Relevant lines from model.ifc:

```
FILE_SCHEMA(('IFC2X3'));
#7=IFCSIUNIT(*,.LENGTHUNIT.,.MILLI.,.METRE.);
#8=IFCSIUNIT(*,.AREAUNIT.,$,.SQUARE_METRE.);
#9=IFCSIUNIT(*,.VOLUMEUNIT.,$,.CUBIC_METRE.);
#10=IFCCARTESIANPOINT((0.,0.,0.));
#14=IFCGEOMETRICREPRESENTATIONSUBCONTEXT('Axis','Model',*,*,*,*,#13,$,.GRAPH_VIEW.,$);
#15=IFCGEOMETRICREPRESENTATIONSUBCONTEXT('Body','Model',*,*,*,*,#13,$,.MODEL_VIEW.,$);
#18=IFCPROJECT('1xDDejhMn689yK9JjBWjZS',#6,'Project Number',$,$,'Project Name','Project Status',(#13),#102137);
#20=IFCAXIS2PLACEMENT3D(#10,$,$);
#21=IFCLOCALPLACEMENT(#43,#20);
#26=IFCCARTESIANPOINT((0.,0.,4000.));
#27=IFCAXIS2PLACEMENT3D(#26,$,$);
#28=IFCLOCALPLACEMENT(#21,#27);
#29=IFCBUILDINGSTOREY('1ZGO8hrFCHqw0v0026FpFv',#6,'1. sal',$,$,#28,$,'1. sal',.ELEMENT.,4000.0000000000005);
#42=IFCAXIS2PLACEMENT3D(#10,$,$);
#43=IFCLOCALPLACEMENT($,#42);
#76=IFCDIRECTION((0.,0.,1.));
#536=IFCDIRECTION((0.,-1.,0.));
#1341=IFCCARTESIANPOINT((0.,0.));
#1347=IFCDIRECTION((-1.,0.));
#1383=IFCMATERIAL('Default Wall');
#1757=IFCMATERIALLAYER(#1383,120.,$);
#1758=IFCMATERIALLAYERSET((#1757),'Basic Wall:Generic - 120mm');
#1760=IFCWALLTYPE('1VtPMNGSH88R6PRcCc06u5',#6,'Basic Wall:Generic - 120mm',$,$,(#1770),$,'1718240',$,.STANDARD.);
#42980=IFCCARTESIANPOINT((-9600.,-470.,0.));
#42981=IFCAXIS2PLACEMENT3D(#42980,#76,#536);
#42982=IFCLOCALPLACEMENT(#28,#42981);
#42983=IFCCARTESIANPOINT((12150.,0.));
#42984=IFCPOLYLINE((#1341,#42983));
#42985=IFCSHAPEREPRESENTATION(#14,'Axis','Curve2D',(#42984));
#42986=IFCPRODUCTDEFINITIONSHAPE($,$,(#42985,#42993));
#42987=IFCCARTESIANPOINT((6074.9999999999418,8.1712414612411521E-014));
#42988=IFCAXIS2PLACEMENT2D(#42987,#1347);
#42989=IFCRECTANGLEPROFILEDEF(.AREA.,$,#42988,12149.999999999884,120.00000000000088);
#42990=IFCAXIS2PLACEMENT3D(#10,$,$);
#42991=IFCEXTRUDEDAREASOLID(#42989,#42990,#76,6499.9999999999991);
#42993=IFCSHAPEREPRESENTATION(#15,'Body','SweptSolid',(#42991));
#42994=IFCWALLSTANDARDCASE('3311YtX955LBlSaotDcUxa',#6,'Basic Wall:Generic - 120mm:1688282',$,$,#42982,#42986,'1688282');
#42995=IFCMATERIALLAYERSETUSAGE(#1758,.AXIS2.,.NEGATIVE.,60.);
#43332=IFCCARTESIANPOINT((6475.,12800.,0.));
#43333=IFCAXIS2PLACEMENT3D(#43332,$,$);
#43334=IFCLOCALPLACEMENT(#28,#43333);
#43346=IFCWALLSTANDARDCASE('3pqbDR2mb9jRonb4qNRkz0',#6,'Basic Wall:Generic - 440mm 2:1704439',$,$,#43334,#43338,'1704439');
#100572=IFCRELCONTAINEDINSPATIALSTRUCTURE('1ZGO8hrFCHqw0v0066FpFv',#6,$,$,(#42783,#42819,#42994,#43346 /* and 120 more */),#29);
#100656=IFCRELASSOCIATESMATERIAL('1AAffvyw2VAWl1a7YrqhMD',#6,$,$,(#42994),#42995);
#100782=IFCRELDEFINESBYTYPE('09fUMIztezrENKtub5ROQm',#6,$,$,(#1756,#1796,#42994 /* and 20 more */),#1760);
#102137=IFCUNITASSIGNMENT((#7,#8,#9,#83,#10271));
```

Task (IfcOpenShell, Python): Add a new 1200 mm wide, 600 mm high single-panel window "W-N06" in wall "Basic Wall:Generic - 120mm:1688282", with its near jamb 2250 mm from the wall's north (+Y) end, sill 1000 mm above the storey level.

```python
import numpy as np
import ifcopenshell
import ifcopenshell.api.feature
import ifcopenshell.api.geometry
import ifcopenshell.api.root
import ifcopenshell.api.spatial
import ifcopenshell.api.type
import ifcopenshell.geom
import ifcopenshell.util.element
import ifcopenshell.util.placement
import ifcopenshell.util.representation
import ifcopenshell.util.shape
import ifcopenshell.util.unit

model = ifcopenshell.open("model.ifc")
unit_scale = ifcopenshell.util.unit.calculate_unit_scale(model)
settings = ifcopenshell.geom.settings()


def volume(element):
    """Net volume in cubic metres, openings subtracted."""
    shape = ifcopenshell.geom.create_shape(settings, element)
    return ifcopenshell.util.shape.get_volume(shape.geometry)


wall = model.by_guid("3311YtX955LBlSaotDcUxa")
storey = ifcopenshell.util.element.get_container(wall, ifc_class="IfcBuildingStorey")
context = ifcopenshell.util.representation.get_context(model, "Model", "Body", "MODEL_VIEW")
before = volume(wall)

width, height, from_end, sill = 1.2, 0.6, 2.25, 1  # metres

# The wall runs along its own X axis, and the end named is its -X end.
wall_shape = ifcopenshell.geom.create_shape(settings, wall)
x, y, z = ifcopenshell.util.shape.get_vertices(wall_shape.geometry).T
start = x.min() + from_end
face, thickness = float(y.min()), float(y.max() - y.min())
wall_matrix = ifcopenshell.util.placement.get_local_placement(wall.ObjectPlacement)
level = ifcopenshell.util.placement.get_local_placement(storey.ObjectPlacement)[2, 3]


def in_wall(x, y):
    """Placement at x, y metres in the wall's axes, at sill height."""
    matrix = wall_matrix.copy()
    matrix[:, 3] = wall_matrix @ np.array([x / unit_scale, y / unit_scale, 0.0, 1.0])
    matrix[2, 3] = level + sill / unit_scale
    return matrix


# Opening: a box that overshoots both wall faces by 50 mm.
opening = ifcopenshell.api.root.create_entity(model, ifc_class="IfcOpeningElement")
box = ifcopenshell.api.geometry.add_wall_representation(
    model, context=context, length=width, height=height, thickness=thickness + 0.1
)
ifcopenshell.api.geometry.assign_representation(model, product=opening, representation=box)
ifcopenshell.api.geometry.edit_object_placement(model, product=opening, matrix=in_wall(start, face - 0.05), is_si=False)
ifcopenshell.api.feature.add_feature(model, feature=opening, element=wall)

window = ifcopenshell.api.root.create_entity(model, ifc_class="IfcWindow", name="W-N06")
window.OverallWidth, window.OverallHeight = width / unit_scale, height / unit_scale
body = ifcopenshell.api.geometry.add_window_representation(
    model,
    context=context,
    overall_width=window.OverallWidth,
    overall_height=window.OverallHeight,
    partition_type="SINGLE_PANEL",
)
ifcopenshell.api.geometry.assign_representation(model, product=window, representation=body)
ifcopenshell.api.spatial.assign_container(model, products=[window], relating_structure=storey)
fills = ifcopenshell.api.feature.add_filling(model, opening=opening, element=window)
fills.OwnerHistory = window.OwnerHistory  # required in IFC2X3

# IFC2X3 keeps the operation on the window style.
style = ifcopenshell.api.root.create_entity(model, ifc_class="IfcWindowStyle", name="W-N06")
style.OperationType, style.ConstructionType = "SINGLE_PANEL", "NOTDEFINED"
style.ParameterTakesPrecedence = style.Sizeable = False
ifcopenshell.api.type.assign_type(model, related_objects=[window], relating_type=style)

# Centre the window in the wall's thickness.
ifcopenshell.api.geometry.edit_object_placement(model, product=window, matrix=in_wall(start, face), is_si=False)
window_shape = ifcopenshell.geom.create_shape(settings, window)
depth = ifcopenshell.util.shape.get_vertices(window_shape.geometry)[:, 1]
offset = face + thickness / 2 - (depth.min() + depth.max()) / 2
ifcopenshell.api.geometry.edit_object_placement(model, product=window, matrix=in_wall(start, offset), is_si=False)

after = volume(wall)

print(f"wall volume {before:.3f} -> {after:.3f} m3")

model.write("model-out.ifc")
```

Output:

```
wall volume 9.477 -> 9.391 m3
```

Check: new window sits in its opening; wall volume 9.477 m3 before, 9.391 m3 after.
